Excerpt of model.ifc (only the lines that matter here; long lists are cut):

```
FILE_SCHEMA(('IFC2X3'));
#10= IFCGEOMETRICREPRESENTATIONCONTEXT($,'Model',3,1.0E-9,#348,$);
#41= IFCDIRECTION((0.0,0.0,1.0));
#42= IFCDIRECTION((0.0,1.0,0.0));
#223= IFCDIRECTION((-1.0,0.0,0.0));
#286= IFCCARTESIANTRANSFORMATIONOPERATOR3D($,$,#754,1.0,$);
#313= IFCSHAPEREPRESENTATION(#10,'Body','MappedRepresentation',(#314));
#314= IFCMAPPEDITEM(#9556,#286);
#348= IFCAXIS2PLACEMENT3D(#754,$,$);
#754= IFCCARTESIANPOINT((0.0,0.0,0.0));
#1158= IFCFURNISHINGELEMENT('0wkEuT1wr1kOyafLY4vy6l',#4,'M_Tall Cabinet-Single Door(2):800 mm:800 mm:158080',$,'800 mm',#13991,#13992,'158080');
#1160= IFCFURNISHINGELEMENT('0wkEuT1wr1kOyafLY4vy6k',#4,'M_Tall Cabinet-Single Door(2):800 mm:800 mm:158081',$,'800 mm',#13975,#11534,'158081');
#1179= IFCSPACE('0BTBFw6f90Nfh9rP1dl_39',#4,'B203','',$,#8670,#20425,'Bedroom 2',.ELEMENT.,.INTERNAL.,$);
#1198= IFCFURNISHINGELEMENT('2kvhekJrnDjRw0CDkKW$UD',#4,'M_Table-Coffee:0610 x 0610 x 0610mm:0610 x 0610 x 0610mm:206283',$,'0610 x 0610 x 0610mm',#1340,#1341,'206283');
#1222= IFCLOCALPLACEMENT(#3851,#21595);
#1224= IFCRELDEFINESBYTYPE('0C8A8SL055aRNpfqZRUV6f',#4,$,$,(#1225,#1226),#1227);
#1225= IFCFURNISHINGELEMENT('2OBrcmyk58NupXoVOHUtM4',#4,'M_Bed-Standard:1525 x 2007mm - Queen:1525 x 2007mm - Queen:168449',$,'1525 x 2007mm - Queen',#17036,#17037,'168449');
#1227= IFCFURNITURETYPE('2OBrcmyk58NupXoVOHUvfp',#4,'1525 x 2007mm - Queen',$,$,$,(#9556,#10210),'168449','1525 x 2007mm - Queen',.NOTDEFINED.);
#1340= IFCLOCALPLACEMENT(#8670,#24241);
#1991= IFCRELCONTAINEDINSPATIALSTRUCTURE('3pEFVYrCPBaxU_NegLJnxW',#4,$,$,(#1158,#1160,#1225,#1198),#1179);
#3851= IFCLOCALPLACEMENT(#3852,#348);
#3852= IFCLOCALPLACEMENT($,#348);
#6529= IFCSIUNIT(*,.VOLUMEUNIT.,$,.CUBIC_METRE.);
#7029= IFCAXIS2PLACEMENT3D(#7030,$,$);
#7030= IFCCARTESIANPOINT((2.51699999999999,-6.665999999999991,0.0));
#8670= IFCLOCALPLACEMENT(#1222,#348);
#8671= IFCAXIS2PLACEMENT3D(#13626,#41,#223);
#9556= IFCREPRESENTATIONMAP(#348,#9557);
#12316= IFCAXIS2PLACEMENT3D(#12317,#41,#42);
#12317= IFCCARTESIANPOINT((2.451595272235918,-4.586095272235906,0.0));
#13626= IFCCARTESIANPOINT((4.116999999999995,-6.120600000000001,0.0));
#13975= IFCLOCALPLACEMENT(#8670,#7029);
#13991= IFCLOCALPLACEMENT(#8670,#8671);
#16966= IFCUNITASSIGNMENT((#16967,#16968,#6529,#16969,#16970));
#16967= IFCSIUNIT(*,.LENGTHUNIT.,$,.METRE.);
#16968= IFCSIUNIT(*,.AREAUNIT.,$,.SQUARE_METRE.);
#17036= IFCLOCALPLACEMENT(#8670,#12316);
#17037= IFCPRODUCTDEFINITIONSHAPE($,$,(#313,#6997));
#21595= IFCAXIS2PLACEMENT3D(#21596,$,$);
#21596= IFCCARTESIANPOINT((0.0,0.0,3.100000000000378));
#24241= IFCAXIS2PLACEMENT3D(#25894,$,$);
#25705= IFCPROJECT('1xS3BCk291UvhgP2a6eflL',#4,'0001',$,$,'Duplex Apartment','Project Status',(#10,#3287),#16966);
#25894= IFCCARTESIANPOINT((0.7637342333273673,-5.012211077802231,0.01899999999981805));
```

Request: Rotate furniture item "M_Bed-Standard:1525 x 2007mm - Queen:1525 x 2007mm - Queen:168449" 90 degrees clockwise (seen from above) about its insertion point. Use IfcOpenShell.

```python
import ifcopenshell
import ifcopenshell.api.geometry
import ifcopenshell.util.placement

model = ifcopenshell.open("model.ifc")

item = model.by_guid("2OBrcmyk58NupXoVOHUtM4")
matrix = ifcopenshell.util.placement.get_local_placement(item.ObjectPlacement)
matrix = matrix @ ifcopenshell.util.placement.rotation(-90, "Z")
ifcopenshell.api.geometry.edit_object_placement(model, product=item, matrix=matrix, is_si=False)

print(ifcopenshell.util.placement.get_local_placement(item.ObjectPlacement).round(3) + 0.0)

model.write("model_rev.ifc")
```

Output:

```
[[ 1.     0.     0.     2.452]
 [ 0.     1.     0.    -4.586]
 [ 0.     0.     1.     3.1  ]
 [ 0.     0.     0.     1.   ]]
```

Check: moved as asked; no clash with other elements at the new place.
